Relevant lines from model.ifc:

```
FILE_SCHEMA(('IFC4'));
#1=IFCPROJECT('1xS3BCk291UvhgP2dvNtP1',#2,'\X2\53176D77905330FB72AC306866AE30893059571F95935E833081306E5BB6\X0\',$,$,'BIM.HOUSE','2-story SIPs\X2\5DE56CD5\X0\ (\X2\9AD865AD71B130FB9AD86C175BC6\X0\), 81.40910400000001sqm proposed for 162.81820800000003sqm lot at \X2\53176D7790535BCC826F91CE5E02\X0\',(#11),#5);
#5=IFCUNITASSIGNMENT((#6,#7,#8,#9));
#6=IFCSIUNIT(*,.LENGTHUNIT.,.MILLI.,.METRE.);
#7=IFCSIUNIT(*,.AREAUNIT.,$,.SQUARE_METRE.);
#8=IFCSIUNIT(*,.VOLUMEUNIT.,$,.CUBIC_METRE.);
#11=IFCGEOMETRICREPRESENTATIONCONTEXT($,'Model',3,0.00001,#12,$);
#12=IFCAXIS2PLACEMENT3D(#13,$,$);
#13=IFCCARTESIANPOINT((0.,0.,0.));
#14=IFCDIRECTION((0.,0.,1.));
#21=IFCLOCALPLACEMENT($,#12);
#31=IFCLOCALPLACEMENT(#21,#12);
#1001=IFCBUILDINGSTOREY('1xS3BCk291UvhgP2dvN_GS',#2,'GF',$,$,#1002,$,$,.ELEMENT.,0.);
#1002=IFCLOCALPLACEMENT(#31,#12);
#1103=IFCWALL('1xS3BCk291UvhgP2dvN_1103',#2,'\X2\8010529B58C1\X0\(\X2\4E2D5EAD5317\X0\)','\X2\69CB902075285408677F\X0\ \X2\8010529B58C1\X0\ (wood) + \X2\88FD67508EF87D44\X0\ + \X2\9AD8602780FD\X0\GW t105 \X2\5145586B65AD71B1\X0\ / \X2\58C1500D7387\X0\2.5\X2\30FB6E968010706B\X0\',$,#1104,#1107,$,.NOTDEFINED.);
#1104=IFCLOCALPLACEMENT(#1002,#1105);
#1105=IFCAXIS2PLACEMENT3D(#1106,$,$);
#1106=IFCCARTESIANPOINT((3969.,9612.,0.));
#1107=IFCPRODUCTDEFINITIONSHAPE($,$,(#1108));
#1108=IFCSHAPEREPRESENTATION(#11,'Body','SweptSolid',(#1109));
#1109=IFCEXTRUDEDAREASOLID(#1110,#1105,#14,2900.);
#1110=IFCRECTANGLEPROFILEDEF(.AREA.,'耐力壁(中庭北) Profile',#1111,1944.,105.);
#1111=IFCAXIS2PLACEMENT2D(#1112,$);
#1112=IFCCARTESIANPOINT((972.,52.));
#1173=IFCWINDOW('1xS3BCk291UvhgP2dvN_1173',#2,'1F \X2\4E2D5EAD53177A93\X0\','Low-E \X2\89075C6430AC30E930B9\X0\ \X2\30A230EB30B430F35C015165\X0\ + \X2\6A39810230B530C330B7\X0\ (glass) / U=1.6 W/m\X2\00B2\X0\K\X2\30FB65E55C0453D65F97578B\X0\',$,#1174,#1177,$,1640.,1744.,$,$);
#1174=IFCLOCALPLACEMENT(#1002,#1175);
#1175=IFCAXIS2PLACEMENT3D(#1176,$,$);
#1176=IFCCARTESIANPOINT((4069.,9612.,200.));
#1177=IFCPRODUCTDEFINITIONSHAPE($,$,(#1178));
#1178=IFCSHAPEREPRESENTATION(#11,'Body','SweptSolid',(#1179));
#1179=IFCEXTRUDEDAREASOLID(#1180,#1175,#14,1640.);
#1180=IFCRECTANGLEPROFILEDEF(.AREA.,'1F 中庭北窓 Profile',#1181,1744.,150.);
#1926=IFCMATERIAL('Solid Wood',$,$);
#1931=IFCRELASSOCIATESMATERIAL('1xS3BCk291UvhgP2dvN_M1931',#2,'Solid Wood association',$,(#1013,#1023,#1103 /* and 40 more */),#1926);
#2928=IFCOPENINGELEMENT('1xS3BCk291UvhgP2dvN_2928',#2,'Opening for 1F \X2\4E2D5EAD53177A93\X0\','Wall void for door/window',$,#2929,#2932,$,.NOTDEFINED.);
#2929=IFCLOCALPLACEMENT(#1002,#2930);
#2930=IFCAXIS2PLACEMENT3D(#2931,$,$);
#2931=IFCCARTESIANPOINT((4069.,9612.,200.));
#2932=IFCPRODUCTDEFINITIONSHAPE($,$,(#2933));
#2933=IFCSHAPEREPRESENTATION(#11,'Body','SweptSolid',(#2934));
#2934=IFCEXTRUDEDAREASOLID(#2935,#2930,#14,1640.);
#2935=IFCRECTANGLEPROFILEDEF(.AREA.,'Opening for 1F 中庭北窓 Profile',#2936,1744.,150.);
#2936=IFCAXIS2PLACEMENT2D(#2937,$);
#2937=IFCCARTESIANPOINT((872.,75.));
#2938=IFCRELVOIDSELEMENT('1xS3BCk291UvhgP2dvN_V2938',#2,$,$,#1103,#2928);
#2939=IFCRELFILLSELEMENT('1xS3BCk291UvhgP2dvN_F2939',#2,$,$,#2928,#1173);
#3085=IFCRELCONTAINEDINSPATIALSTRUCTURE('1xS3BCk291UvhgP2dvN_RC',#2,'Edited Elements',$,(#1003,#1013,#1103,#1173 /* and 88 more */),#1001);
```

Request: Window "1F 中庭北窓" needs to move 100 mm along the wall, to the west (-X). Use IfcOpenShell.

```python
import ifcopenshell
import ifcopenshell.api.geometry
import ifcopenshell.util.placement

model = ifcopenshell.open("model.ifc")

window = model.by_guid("1xS3BCk291UvhgP2dvN_1173")
opening = window.FillsVoids[0].RelatingOpeningElement
wall = opening.VoidsElements[0].RelatingBuildingElement

wall_matrix = ifcopenshell.util.placement.get_local_placement(wall.ObjectPlacement)
shift = wall_matrix[:3, 0] * -100.0
before = ifcopenshell.util.placement.get_local_placement(window.ObjectPlacement)[:3, 3].copy()

# The window is not placed relative to its opening, so move both.
for product in (opening, window):
    matrix = ifcopenshell.util.placement.get_local_placement(product.ObjectPlacement)
    matrix[:3, 3] += shift
    ifcopenshell.api.geometry.edit_object_placement(model, product=product, matrix=matrix, is_si=False)

after = ifcopenshell.util.placement.get_local_placement(window.ObjectPlacement)[:3, 3]
print("window moved by", (after - before).round(3) + 0.0)

model.write("model_v2.ifc")
```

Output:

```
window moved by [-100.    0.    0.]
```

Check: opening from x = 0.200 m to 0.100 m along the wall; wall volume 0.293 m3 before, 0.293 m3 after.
